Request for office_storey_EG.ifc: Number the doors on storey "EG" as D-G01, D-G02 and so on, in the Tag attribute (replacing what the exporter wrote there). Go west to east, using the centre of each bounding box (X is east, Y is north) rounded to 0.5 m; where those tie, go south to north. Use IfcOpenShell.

First a look at what the model holds.

```python
import ifcopenshell
import ifcopenshell.util.element
import ifcopenshell.util.placement

model = ifcopenshell.open("office_storey_EG.ifc")
print(model.schema)
storey = next(s for s in model.by_type("IfcBuildingStorey") if s.Name == "EG")
doors = [e for e in ifcopenshell.util.element.get_decomposition(storey) if e.is_a("IfcDoor")]
for e in sorted(doors, key=lambda e: e.id()):
    origin = ifcopenshell.util.placement.get_local_placement(e.ObjectPlacement)[:3, 3]
    print(e.id(), e.Tag, e.Name, origin.round(2) + 0.0, sep=" | ")
```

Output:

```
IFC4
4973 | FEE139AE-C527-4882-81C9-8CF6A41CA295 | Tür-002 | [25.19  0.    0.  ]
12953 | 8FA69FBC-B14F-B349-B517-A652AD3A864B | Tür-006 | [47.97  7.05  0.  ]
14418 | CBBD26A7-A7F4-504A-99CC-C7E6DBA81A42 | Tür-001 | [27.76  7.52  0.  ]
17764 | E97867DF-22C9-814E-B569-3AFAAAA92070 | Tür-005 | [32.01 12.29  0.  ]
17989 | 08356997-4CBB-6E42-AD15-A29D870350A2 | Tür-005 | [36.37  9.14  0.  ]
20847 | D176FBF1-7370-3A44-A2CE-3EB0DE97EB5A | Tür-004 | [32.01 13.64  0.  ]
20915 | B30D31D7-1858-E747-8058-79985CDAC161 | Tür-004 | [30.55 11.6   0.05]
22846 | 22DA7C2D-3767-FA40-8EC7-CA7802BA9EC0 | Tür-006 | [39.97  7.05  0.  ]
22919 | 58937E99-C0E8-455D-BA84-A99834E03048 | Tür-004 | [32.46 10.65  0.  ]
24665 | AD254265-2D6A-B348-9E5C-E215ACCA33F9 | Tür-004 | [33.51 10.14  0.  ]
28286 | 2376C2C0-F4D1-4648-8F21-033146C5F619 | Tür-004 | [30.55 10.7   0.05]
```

```python
import ifcopenshell
import ifcopenshell.geom
import ifcopenshell.util.element
import ifcopenshell.util.shape

model = ifcopenshell.open("office_storey_EG.ifc")
settings = ifcopenshell.geom.settings()
settings.set("use-world-coords", True)


def centre(element):
    shape = ifcopenshell.geom.create_shape(settings, element)
    return ifcopenshell.util.shape.get_bbox_centroid(shape.geometry)


storey = next(s for s in model.by_type("IfcBuildingStorey") if s.Name == "EG")
doors = [e for e in ifcopenshell.util.element.get_decomposition(storey) if e.is_a("IfcDoor")]

# Insertion points can sit at a corner or the storey origin, so sort by the geometry (in metres).
centres = {e: centre(e) for e in doors}
doors.sort(key=lambda e: (round(centres[e][0] / 0.5), centres[e][1]))

for i, e in enumerate(doors, start=1):
    number = f"D-G{i:02d}"
    e.Tag = number
    print(e.id(), number)

model.write("office_storey_EG-out.ifc")
```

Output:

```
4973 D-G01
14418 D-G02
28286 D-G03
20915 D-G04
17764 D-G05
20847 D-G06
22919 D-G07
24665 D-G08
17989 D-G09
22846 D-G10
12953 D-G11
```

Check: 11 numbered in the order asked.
